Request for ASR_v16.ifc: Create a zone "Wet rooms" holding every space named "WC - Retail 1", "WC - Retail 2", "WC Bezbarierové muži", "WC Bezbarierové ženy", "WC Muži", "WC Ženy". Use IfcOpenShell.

First a look at what the model holds.

```python
import ifcopenshell

model = ifcopenshell.open("ASR_v16.ifc")
print(model.schema)
seen = {}
for space in model.by_type("IfcSpace"):
    seen[space.LongName] = seen.get(space.LongName, 0) + 1
for name, count in sorted(seen.items(), key=str):
    print(count, "x", name)
print("zones:", [z.Name for z in model.by_type("IfcZone")][:20])
```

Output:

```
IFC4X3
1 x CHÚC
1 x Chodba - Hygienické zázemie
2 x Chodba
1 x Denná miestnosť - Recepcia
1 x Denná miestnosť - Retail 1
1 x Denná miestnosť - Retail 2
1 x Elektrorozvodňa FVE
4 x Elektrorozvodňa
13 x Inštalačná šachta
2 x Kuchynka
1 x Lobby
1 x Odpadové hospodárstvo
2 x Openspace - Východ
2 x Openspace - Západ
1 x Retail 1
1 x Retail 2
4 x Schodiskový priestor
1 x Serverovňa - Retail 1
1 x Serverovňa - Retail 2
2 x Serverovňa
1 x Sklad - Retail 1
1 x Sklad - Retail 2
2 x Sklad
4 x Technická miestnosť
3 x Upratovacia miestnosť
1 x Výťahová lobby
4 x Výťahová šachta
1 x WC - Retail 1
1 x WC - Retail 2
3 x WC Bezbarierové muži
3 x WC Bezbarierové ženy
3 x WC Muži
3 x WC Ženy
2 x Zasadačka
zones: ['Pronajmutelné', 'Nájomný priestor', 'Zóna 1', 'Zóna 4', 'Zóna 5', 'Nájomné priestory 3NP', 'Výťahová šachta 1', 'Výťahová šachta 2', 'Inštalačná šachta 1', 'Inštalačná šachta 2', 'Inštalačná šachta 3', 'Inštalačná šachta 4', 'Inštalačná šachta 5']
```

```python
import ifcopenshell
import ifcopenshell.api.group
import ifcopenshell.api.root

model = ifcopenshell.open("ASR_v16.ifc")

names = {"WC - Retail 1", "WC - Retail 2", "WC Bezbarierové muži", "WC Bezbarierové ženy", "WC Muži", "WC Ženy"}
spaces = [s for s in model.by_type("IfcSpace") if s.LongName in names]

zone = ifcopenshell.api.root.create_entity(model, ifc_class="IfcZone", name="Wet rooms")
ifcopenshell.api.group.assign_group(model, products=spaces, group=zone)
print(len(spaces), "spaces in", zone.Name)

model.write("ASR_v16-out.ifc")
```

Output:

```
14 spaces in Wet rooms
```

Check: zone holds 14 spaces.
